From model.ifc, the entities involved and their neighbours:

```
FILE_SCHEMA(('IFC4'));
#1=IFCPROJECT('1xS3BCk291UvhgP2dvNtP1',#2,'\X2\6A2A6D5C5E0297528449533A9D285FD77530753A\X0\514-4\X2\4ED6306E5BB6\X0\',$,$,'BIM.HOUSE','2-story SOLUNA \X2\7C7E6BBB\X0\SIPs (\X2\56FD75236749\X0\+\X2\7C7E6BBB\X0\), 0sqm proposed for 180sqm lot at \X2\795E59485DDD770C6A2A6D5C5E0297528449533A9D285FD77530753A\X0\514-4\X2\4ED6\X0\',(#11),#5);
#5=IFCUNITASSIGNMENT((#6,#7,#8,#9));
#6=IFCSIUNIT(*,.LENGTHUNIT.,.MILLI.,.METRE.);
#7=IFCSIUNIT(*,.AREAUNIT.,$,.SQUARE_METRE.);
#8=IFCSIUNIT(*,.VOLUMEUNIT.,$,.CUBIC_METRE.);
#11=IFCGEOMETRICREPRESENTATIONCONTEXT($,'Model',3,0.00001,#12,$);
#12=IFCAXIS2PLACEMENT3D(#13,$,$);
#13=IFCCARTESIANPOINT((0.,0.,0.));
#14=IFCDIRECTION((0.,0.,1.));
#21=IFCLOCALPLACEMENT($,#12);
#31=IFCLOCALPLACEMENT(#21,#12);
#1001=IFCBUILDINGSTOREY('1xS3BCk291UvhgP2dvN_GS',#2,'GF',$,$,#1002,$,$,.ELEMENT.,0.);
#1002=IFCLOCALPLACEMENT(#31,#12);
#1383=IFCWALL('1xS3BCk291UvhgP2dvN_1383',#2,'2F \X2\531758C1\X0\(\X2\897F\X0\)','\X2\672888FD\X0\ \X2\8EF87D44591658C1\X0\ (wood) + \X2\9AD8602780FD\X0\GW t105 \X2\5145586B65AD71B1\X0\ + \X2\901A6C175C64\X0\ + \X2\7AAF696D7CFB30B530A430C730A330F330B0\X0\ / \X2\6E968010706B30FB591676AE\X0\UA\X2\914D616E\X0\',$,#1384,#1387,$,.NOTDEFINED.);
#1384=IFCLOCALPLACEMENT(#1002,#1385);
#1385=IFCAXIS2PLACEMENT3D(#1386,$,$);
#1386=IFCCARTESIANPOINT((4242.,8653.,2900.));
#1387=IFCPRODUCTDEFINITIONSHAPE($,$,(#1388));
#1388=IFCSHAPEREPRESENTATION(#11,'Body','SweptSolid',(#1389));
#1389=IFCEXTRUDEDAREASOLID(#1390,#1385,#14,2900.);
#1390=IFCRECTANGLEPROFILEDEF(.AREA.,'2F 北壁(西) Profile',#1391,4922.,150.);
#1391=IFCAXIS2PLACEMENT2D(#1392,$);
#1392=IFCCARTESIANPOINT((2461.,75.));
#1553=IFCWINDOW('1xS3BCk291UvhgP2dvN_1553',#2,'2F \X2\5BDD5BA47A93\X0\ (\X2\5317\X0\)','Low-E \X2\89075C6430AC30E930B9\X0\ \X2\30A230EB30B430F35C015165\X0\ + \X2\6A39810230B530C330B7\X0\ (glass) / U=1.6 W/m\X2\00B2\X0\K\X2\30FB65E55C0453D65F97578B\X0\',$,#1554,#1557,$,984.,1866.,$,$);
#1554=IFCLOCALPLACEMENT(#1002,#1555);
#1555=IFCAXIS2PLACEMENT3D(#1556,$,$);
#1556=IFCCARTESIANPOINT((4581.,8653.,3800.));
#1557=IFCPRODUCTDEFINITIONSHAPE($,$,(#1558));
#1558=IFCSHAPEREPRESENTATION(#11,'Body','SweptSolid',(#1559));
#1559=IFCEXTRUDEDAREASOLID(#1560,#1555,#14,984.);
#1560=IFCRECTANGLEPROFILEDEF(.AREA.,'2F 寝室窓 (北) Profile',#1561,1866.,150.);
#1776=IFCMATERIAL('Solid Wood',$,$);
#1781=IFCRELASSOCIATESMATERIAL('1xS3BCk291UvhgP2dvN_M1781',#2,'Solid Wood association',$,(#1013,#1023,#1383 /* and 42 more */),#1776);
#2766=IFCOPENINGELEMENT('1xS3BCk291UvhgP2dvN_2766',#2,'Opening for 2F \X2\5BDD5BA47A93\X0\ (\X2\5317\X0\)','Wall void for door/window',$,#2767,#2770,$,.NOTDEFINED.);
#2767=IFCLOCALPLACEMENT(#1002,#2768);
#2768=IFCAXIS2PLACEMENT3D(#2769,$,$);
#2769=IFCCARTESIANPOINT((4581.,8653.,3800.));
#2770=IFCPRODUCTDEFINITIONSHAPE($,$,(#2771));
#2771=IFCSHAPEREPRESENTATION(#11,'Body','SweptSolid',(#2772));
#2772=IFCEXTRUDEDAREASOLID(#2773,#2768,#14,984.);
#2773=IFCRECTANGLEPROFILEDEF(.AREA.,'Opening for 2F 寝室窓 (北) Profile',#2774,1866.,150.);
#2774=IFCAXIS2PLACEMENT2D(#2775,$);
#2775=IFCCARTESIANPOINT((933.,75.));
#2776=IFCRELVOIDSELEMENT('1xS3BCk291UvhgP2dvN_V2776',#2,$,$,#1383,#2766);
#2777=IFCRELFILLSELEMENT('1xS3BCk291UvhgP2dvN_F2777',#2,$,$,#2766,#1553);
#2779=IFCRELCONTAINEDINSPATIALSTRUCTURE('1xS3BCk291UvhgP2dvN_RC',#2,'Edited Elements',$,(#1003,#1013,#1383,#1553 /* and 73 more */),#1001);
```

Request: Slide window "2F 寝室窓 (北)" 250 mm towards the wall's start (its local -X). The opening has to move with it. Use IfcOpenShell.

```python
import ifcopenshell
import ifcopenshell.api.geometry
import ifcopenshell.util.placement

model = ifcopenshell.open("model.ifc")

window = model.by_guid("1xS3BCk291UvhgP2dvN_1553")
opening = window.FillsVoids[0].RelatingOpeningElement
wall = opening.VoidsElements[0].RelatingBuildingElement

wall_matrix = ifcopenshell.util.placement.get_local_placement(wall.ObjectPlacement)
shift = wall_matrix[:3, 0] * -250.0
before = ifcopenshell.util.placement.get_local_placement(window.ObjectPlacement)[:3, 3].copy()

# The window is not placed relative to its opening, so move both.
for product in (opening, window):
    matrix = ifcopenshell.util.placement.get_local_placement(product.ObjectPlacement)
    matrix[:3, 3] += shift
    ifcopenshell.api.geometry.edit_object_placement(model, product=product, matrix=matrix, is_si=False)

after = ifcopenshell.util.placement.get_local_placement(window.ObjectPlacement)[:3, 3]
print("window moved by", (after - before).round(3) + 0.0)

model.write("model_edited.ifc")
```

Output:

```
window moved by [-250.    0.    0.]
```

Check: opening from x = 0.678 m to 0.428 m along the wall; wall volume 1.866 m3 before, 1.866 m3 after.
